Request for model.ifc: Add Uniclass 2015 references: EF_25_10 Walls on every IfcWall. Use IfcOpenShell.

First a look at what the model holds.

```python
import ifcopenshell

model = ifcopenshell.open("model.ifc")
print(model.schema)
print("classifications:", [c.Name for c in model.by_type("IfcClassification")])
for ifc_class in ("IfcDoor", "IfcRoof", "IfcStair", "IfcWall", "IfcWindow"):
    print(ifc_class, len(model.by_type(ifc_class)))
```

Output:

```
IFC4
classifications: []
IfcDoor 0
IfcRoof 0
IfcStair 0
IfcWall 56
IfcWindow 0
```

```python
import ifcopenshell
import ifcopenshell.api.classification

model = ifcopenshell.open("model.ifc")

system = ifcopenshell.api.classification.add_classification(model, classification="Uniclass 2015")

codes = {
    "IfcWall": ("EF_25_10", "Walls"),
}
for ifc_class, (code, name) in codes.items():
    products = model.by_type(ifc_class)
    ifcopenshell.api.classification.add_reference(
        model, products=products, classification=system, identification=code, name=name
    )
    print(code, len(products))

model.write("model_v2.ifc")
```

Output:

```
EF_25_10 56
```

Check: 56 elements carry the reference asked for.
